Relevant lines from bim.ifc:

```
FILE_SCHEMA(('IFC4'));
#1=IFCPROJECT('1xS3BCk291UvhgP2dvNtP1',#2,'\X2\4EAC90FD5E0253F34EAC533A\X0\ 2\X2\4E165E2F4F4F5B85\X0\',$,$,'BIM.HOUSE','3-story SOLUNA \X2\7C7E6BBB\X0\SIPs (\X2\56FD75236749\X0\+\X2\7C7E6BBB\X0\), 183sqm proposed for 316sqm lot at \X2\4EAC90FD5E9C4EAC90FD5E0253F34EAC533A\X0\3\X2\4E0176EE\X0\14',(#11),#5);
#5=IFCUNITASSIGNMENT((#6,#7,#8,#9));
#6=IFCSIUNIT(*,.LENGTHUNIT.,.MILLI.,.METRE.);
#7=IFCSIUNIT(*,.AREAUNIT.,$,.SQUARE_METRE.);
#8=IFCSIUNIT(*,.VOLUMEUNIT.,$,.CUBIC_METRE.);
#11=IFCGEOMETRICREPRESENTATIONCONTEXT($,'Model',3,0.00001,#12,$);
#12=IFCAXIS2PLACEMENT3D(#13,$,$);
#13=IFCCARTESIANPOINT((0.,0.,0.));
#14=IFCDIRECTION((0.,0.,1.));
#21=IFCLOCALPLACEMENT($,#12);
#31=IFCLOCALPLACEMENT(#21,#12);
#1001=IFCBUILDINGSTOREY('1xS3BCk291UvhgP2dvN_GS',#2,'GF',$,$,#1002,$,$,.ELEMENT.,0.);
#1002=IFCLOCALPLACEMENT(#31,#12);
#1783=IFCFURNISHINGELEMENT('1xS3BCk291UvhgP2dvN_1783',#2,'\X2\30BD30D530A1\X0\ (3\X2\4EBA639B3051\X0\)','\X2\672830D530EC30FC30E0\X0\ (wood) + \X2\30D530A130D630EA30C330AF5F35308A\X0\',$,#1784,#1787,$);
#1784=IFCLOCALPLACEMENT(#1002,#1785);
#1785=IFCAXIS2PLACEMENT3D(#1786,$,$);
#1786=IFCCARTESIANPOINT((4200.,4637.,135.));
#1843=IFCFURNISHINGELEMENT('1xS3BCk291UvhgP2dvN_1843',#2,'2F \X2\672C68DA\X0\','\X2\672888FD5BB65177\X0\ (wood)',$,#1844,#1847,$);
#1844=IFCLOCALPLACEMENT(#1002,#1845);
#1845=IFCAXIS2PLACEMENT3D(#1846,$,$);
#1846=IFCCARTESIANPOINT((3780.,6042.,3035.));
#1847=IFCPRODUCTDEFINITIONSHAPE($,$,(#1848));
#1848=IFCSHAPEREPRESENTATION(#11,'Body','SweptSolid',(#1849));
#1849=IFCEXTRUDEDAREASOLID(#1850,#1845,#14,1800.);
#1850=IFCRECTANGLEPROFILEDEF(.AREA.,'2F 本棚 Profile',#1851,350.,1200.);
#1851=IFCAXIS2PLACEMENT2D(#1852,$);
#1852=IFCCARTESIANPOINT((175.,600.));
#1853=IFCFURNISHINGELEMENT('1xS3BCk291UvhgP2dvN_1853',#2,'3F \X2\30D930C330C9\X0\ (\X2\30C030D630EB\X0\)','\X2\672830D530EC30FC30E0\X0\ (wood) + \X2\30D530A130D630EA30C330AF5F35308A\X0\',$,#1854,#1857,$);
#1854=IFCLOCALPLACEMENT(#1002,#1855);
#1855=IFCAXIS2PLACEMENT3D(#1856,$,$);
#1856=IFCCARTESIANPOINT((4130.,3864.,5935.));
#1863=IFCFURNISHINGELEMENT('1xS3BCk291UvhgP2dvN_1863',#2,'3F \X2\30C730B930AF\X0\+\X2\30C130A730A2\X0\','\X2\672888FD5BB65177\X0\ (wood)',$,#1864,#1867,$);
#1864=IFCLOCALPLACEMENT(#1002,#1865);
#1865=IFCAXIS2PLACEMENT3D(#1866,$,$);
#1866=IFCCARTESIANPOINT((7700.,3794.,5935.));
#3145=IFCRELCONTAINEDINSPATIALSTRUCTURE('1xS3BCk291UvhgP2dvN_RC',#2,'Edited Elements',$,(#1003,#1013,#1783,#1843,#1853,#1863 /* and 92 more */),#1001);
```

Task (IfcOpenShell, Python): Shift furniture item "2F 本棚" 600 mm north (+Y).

```python
import ifcopenshell
import ifcopenshell.api.geometry
import ifcopenshell.util.placement
import ifcopenshell.util.unit

model = ifcopenshell.open("bim.ifc")
unit_scale = ifcopenshell.util.unit.calculate_unit_scale(model)

item = model.by_guid("1xS3BCk291UvhgP2dvN_1843")
matrix = ifcopenshell.util.placement.get_local_placement(item.ObjectPlacement)
matrix[1, 3] += 0.6 / unit_scale
ifcopenshell.api.geometry.edit_object_placement(model, product=item, matrix=matrix, is_si=False)

print(ifcopenshell.util.placement.get_local_placement(item.ObjectPlacement).round(3) + 0.0)

model.write("bim_v2.ifc")
```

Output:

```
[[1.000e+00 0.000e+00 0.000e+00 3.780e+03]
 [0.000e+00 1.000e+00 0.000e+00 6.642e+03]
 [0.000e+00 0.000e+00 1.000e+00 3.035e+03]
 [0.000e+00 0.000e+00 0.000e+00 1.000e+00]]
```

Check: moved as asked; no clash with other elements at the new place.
